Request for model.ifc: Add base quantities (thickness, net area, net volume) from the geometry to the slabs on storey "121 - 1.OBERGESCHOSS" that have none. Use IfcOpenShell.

First a look at what the model holds.

```python
import ifcopenshell
import ifcopenshell.util.element
import ifcopenshell.util.unit

model = ifcopenshell.open("model.ifc")
print(model.schema)
for unit_type in ("LENGTHUNIT", "AREAUNIT", "VOLUMEUNIT"):
    print(unit_type, ifcopenshell.util.unit.calculate_unit_scale(model, unit_type))
storey = next(s for s in model.by_type("IfcBuildingStorey") if s.Name == "121 - 1.OBERGESCHOSS")
slabs = [e for e in ifcopenshell.util.element.get_decomposition(storey) if e.is_a("IfcSlab")]
for e in sorted(slabs, key=lambda e: e.id()):
    print(e.id(), e.is_a(), e.Name, list(ifcopenshell.util.element.get_psets(e, qtos_only=True)), sep=" | ")
```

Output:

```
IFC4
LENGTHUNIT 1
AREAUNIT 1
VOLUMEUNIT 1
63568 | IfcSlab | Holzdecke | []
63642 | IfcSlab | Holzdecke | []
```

```python
import ifcopenshell
import ifcopenshell.api.pset
import ifcopenshell.geom
import ifcopenshell.util.element
import ifcopenshell.util.shape
import ifcopenshell.util.unit

model = ifcopenshell.open("model.ifc")
unit_scale = ifcopenshell.util.unit.calculate_unit_scale(model)
area_scale = ifcopenshell.util.unit.calculate_unit_scale(model, "AREAUNIT")
volume_scale = ifcopenshell.util.unit.calculate_unit_scale(model, "VOLUMEUNIT")
settings = ifcopenshell.geom.settings()

storey = next(s for s in model.by_type("IfcBuildingStorey") if s.Name == "121 - 1.OBERGESCHOSS")
slabs = [e for e in ifcopenshell.util.element.get_decomposition(storey) if e.is_a("IfcSlab")]

for e in sorted(slabs, key=lambda e: e.id()):
    if ifcopenshell.util.element.get_psets(e, qtos_only=True, should_inherit=False):
        continue
    # Geometry comes back in metres, in the element's own axes.
    shape = ifcopenshell.geom.create_shape(settings, e)
    values = {
        "Width": ifcopenshell.util.shape.get_z(shape.geometry) / unit_scale,
        "NetArea": ifcopenshell.util.shape.get_footprint_area(shape.geometry) / area_scale,
        "NetVolume": ifcopenshell.util.shape.get_volume(shape.geometry) / volume_scale,
    }
    qto = ifcopenshell.api.pset.add_qto(model, product=e, name="Qto_SlabBaseQuantities")
    ifcopenshell.api.pset.edit_qto(model, qto=qto, properties=values)
    print(e.id(), {k: round(v, 3) for k, v in values.items()})

model.write("model_updated.ifc")
```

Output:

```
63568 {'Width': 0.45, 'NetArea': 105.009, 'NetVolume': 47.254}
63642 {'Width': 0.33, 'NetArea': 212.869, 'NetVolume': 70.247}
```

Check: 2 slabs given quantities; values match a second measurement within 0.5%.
